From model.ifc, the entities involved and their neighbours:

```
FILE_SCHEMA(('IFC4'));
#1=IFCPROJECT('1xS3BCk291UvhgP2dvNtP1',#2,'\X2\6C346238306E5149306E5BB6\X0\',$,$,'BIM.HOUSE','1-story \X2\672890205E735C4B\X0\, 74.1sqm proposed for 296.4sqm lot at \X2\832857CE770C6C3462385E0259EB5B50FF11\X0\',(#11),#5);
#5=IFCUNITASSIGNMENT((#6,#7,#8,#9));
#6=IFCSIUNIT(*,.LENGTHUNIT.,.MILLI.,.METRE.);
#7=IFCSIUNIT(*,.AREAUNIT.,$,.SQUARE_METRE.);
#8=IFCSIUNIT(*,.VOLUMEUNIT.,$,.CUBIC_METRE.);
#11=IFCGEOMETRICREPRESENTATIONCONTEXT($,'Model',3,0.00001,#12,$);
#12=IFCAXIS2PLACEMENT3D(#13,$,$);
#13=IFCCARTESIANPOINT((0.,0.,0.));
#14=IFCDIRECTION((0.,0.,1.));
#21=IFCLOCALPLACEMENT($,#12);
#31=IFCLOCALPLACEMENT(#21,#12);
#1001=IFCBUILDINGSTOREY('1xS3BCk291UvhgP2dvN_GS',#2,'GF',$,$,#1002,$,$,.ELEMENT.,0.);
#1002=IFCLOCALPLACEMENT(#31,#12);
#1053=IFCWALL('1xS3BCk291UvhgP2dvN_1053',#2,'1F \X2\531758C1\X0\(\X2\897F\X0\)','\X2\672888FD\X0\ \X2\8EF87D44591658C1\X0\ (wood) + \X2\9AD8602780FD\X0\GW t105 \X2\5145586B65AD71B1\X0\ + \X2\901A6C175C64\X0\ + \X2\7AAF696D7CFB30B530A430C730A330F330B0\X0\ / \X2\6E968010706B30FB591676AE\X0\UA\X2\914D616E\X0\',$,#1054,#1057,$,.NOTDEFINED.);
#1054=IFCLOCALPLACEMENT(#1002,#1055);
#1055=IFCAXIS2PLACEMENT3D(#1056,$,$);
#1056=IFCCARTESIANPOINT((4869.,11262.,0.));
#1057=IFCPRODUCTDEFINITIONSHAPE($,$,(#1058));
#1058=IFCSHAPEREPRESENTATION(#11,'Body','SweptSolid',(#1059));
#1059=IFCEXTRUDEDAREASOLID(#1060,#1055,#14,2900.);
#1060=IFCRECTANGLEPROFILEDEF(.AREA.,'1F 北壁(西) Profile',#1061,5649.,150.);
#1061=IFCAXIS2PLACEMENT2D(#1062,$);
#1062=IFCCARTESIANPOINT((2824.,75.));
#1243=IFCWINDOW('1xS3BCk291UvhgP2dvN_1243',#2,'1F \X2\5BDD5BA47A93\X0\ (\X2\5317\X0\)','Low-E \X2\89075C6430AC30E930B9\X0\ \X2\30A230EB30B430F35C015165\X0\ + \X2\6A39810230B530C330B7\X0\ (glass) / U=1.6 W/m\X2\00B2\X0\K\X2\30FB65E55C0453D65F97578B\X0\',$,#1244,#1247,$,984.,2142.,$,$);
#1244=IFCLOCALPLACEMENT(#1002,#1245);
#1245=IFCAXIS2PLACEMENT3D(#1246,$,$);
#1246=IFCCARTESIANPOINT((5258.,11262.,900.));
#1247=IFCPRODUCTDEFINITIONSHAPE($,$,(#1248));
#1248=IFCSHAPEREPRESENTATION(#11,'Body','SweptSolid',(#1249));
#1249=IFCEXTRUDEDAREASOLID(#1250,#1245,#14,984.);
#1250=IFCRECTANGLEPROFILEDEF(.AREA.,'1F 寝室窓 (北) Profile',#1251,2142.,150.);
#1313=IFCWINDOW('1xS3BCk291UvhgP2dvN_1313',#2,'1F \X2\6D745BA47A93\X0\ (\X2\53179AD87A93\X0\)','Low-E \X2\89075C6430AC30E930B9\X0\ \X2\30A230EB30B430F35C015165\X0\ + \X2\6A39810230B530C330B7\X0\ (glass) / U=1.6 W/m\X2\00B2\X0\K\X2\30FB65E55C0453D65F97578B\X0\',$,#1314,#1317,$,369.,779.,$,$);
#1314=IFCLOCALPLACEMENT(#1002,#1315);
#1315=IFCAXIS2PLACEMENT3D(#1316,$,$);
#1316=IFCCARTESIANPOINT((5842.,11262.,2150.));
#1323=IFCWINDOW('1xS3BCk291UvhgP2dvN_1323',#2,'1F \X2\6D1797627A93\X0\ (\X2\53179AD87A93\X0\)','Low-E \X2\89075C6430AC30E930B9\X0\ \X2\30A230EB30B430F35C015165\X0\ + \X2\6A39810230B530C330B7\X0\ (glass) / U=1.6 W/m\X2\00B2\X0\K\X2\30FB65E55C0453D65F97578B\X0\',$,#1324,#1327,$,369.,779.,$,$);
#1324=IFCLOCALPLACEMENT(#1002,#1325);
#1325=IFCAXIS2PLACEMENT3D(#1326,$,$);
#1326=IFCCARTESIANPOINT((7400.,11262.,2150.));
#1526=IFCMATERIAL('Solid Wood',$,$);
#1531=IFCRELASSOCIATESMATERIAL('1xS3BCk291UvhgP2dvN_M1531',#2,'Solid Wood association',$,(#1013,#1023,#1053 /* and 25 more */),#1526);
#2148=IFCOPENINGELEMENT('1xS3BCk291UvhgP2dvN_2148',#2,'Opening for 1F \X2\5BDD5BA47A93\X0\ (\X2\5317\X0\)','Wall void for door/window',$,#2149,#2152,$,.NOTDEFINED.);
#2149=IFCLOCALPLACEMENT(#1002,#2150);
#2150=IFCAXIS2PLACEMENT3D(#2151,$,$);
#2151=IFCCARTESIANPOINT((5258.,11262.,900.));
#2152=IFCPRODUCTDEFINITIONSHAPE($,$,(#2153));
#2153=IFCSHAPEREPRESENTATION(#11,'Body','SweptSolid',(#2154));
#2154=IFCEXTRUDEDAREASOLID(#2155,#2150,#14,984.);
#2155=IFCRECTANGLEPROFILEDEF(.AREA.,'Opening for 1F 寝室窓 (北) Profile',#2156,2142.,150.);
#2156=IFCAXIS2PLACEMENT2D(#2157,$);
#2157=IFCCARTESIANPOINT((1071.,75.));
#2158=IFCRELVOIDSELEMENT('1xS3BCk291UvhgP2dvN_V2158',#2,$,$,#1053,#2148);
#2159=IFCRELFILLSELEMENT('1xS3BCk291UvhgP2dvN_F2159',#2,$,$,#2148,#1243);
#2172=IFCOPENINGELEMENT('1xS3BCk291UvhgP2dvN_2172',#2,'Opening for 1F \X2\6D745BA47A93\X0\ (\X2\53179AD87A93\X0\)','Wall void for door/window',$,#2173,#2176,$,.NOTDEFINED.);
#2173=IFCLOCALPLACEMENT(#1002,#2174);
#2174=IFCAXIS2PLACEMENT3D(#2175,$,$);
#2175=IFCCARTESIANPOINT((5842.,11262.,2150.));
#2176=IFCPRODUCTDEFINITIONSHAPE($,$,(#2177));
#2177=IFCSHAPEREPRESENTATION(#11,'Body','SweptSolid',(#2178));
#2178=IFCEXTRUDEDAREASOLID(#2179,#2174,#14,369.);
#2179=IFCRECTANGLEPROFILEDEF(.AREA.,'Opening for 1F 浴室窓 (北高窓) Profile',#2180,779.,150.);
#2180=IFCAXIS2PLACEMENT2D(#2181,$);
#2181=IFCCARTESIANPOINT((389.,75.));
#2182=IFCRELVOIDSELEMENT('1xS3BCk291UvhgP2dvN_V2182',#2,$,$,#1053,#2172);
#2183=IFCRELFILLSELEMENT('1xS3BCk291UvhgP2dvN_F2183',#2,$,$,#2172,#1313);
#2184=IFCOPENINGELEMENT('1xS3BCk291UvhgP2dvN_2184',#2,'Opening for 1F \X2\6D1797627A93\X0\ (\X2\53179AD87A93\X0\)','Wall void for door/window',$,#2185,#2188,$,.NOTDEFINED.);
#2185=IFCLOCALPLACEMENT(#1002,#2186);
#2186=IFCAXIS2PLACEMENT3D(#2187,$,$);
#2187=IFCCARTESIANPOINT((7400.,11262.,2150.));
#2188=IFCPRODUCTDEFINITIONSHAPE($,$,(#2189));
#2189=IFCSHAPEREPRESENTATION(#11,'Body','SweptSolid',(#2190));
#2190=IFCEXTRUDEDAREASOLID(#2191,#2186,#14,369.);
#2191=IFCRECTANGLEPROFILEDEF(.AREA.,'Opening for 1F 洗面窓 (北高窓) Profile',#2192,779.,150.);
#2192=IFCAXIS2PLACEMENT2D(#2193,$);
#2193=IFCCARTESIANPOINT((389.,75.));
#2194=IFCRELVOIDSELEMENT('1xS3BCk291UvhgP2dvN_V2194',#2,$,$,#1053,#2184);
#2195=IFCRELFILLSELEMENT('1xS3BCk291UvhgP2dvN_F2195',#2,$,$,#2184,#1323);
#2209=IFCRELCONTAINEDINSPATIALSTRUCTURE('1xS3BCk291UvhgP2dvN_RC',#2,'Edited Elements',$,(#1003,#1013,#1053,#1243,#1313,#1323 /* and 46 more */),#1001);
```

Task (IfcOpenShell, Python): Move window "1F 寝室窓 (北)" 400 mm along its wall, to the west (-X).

```python
import ifcopenshell
import ifcopenshell.api.geometry
import ifcopenshell.util.placement

model = ifcopenshell.open("model.ifc")

window = model.by_id(1243)
opening = window.FillsVoids[0].RelatingOpeningElement
wall = opening.VoidsElements[0].RelatingBuildingElement

wall_matrix = ifcopenshell.util.placement.get_local_placement(wall.ObjectPlacement)
shift = wall_matrix[:3, 0] * -400.0
before = ifcopenshell.util.placement.get_local_placement(window.ObjectPlacement)[:3, 3].copy()

# The window is not placed relative to its opening, so move both.
for product in (opening, window):
    matrix = ifcopenshell.util.placement.get_local_placement(product.ObjectPlacement)
    matrix[:3, 3] += shift
    ifcopenshell.api.geometry.edit_object_placement(model, product=product, matrix=matrix, is_si=False)

after = ifcopenshell.util.placement.get_local_placement(window.ObjectPlacement)[:3, 3]
print("window moved by", (after - before).round(3) + 0.0)

model.write("model_edited.ifc")
```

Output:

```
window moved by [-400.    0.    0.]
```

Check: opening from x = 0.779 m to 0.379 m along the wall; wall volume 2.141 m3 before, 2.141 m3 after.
